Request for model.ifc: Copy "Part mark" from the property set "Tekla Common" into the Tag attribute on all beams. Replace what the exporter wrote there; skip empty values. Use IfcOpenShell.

First a look at what the model holds.

```python
import ifcopenshell
import ifcopenshell.util.element

model = ifcopenshell.open("model.ifc")
print(model.schema)
beams = model.by_type("IfcBeam")
print(len(beams), "beams")
for e in beams[:8]:
    source = ifcopenshell.util.element.get_pset(e, "Tekla Common", "Part mark")
    target = e.Tag
    print(e.id(), repr(source), repr(target), sep=" | ")
```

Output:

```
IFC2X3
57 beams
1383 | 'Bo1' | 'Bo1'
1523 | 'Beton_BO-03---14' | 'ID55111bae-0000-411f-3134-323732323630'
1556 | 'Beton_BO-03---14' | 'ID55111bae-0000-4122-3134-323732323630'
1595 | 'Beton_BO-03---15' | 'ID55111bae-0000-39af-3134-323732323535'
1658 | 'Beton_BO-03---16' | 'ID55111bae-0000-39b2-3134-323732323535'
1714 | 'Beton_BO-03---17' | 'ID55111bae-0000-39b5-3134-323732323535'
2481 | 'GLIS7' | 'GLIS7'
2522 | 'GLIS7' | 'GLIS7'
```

```python
import ifcopenshell
import ifcopenshell.util.element

model = ifcopenshell.open("model.ifc")

count = 0
for e in model.by_type("IfcBeam"):
    value = ifcopenshell.util.element.get_pset(e, "Tekla Common", "Part mark")
    current = e.Tag
    if not value or not value.strip() or current == value:
        continue
    e.Tag = value
    count += 1

print(count, "beams updated")

model.write("model_v2.ifc")
```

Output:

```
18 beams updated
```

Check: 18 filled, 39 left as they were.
